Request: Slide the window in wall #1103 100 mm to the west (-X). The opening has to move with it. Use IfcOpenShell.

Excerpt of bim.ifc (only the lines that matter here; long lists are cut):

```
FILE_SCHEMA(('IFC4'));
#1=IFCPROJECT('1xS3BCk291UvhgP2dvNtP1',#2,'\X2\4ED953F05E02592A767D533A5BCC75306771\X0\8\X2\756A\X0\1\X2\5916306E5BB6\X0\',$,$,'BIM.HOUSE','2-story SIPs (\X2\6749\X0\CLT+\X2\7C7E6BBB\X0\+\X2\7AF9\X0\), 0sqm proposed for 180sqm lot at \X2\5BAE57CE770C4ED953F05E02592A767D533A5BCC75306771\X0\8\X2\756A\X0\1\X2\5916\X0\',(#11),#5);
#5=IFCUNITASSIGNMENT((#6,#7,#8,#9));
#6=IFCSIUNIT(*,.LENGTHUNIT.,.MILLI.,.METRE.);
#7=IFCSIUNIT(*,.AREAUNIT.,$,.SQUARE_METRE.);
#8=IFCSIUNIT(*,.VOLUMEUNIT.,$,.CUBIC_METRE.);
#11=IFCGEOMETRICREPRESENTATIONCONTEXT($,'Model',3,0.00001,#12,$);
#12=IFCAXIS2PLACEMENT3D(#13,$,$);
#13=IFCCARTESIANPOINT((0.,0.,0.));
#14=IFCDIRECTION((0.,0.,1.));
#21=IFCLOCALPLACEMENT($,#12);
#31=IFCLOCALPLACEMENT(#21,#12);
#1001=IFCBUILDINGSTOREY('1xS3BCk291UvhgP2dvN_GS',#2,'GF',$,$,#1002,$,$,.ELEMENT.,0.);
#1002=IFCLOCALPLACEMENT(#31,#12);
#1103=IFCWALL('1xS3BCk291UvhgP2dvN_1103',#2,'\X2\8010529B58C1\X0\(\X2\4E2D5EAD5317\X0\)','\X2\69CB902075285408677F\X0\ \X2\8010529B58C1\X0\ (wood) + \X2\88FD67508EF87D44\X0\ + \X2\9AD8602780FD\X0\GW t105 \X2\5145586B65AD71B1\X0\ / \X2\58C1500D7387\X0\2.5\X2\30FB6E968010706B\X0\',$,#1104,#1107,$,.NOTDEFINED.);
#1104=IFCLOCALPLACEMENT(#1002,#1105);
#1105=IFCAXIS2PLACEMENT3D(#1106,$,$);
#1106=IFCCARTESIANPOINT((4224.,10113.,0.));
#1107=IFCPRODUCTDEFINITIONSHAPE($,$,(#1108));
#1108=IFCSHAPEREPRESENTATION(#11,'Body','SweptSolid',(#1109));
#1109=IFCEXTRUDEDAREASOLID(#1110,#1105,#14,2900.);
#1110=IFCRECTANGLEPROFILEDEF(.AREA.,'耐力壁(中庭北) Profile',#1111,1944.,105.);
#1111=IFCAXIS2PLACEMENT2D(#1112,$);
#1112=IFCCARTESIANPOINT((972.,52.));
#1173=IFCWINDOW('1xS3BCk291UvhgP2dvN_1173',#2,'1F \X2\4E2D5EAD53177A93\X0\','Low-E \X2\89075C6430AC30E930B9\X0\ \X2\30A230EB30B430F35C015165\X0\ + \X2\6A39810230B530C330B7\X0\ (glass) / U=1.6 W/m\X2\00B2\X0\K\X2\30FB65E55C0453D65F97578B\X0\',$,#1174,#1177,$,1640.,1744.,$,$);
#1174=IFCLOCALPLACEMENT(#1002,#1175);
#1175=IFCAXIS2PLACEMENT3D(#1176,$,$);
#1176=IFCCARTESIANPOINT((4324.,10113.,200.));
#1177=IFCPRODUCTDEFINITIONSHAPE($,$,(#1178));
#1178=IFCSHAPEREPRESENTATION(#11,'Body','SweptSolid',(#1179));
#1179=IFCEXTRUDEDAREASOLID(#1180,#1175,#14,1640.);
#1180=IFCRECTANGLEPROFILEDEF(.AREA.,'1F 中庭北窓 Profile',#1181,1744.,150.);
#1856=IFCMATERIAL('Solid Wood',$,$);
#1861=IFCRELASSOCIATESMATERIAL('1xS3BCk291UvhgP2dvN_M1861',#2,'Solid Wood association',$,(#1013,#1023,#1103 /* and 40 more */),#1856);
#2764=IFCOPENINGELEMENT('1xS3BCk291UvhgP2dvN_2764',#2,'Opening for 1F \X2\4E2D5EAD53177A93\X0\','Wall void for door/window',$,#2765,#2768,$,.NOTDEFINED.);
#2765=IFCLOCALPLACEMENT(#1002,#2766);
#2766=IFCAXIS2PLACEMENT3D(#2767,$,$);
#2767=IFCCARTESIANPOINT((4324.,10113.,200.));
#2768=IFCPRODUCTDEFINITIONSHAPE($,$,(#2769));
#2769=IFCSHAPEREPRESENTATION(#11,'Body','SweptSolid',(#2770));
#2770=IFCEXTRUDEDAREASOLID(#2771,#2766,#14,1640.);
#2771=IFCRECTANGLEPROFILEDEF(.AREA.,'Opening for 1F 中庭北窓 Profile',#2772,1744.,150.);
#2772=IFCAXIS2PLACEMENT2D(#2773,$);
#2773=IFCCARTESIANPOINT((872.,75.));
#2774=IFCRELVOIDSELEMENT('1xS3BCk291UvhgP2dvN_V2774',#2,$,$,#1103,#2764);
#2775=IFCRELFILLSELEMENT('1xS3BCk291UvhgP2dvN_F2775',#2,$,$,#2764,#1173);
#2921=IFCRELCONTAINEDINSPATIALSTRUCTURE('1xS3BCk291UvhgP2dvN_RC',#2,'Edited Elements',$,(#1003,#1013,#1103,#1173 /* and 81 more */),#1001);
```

```python
import ifcopenshell
import ifcopenshell.api.geometry
import ifcopenshell.util.placement

model = ifcopenshell.open("bim.ifc")

window = model.by_guid("1xS3BCk291UvhgP2dvN_1173")
opening = window.FillsVoids[0].RelatingOpeningElement
wall = opening.VoidsElements[0].RelatingBuildingElement

wall_matrix = ifcopenshell.util.placement.get_local_placement(wall.ObjectPlacement)
shift = wall_matrix[:3, 0] * -100.0
before = ifcopenshell.util.placement.get_local_placement(window.ObjectPlacement)[:3, 3].copy()

# The window is not placed relative to its opening, so move both.
for product in (opening, window):
    matrix = ifcopenshell.util.placement.get_local_placement(product.ObjectPlacement)
    matrix[:3, 3] += shift
    ifcopenshell.api.geometry.edit_object_placement(model, product=product, matrix=matrix, is_si=False)

after = ifcopenshell.util.placement.get_local_placement(window.ObjectPlacement)[:3, 3]
print("window moved by", (after - before).round(3) + 0.0)

model.write("bim_edited.ifc")
```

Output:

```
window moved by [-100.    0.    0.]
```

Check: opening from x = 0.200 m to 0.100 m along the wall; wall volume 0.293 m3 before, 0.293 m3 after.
